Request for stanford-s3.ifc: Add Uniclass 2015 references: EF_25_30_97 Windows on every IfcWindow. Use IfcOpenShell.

First a look at what the model holds.

```python
import ifcopenshell

model = ifcopenshell.open("stanford-s3.ifc")
print(model.schema)
print("classifications:", [c.Name for c in model.by_type("IfcClassification")])
for ifc_class in ("IfcDoor", "IfcRoof", "IfcStair", "IfcWall", "IfcWindow"):
    print(ifc_class, len(model.by_type(ifc_class)))
```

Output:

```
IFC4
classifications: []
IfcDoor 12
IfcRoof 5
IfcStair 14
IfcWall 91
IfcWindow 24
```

```python
import ifcopenshell
import ifcopenshell.api.classification

model = ifcopenshell.open("stanford-s3.ifc")

system = ifcopenshell.api.classification.add_classification(model, classification="Uniclass 2015")

codes = {
    "IfcWindow": ("EF_25_30_97", "Windows"),
}
for ifc_class, (code, name) in codes.items():
    products = model.by_type(ifc_class)
    ifcopenshell.api.classification.add_reference(
        model, products=products, classification=system, identification=code, name=name
    )
    print(code, len(products))

model.write("stanford-s3_v2.ifc")
```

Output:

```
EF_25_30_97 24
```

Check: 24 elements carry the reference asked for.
